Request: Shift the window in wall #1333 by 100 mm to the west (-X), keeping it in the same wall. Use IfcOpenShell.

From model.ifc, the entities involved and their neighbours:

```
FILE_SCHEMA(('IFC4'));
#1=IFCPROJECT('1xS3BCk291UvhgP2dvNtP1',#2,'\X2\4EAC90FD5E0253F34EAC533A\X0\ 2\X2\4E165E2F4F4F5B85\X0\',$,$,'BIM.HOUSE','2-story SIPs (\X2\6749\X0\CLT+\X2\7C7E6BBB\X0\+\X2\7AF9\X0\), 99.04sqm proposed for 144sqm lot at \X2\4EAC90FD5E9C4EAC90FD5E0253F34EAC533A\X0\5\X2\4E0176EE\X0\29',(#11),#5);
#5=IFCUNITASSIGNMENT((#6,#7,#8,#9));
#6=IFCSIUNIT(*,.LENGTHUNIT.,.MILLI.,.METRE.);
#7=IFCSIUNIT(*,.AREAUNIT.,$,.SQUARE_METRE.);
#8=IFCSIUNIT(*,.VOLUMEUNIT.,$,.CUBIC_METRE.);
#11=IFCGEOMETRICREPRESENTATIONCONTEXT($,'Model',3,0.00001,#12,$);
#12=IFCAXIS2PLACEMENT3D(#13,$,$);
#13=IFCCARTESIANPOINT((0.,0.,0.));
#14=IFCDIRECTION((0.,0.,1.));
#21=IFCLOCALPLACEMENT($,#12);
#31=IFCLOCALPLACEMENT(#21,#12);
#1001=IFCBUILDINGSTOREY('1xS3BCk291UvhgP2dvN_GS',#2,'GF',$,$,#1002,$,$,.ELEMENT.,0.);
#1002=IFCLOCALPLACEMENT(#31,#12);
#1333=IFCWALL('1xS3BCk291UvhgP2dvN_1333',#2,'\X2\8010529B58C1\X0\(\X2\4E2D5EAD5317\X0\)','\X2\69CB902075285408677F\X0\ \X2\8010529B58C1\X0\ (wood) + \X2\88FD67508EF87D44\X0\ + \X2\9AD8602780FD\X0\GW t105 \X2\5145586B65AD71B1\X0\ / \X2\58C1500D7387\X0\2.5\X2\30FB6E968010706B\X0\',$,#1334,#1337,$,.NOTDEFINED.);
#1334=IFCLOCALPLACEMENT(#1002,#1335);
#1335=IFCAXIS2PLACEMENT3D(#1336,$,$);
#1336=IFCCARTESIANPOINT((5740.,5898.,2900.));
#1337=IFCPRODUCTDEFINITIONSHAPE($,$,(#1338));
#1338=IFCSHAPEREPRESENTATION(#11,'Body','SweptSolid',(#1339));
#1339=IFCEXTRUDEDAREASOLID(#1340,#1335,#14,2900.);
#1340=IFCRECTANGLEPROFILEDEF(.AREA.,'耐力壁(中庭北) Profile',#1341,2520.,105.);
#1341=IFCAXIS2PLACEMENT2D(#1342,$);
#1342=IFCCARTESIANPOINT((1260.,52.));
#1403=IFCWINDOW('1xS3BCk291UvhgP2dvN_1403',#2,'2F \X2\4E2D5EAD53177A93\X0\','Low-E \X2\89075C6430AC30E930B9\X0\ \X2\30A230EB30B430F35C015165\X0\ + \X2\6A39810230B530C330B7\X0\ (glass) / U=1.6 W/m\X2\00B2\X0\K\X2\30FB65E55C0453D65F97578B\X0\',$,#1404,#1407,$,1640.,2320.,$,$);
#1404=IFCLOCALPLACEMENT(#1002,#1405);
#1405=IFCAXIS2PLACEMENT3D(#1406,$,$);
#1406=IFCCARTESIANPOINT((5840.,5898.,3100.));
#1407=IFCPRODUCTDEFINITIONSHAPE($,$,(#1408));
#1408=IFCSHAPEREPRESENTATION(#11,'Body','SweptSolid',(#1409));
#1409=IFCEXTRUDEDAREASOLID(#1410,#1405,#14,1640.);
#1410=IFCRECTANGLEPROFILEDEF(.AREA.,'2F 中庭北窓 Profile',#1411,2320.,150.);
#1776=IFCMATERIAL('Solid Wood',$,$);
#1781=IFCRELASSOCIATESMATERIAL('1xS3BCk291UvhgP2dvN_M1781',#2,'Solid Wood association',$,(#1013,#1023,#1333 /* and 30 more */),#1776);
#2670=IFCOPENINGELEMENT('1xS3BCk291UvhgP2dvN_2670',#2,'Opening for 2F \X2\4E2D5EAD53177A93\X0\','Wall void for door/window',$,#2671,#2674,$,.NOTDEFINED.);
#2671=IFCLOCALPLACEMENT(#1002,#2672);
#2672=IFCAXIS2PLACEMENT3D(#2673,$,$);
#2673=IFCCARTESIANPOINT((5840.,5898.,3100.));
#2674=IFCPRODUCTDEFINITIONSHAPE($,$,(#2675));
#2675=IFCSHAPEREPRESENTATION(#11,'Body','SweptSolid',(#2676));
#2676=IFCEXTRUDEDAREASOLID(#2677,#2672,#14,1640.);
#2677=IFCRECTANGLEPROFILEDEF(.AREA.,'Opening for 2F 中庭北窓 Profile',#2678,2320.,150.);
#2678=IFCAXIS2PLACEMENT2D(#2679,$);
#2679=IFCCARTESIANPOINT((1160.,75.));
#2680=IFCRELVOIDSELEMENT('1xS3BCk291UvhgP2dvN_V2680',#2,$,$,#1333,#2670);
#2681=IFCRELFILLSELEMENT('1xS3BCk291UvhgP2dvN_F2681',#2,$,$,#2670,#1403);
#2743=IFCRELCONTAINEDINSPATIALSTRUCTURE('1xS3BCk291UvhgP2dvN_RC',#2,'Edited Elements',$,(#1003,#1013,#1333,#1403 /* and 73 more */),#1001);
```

```python
import ifcopenshell
import ifcopenshell.api.geometry
import ifcopenshell.util.placement
import ifcopenshell.util.unit

model = ifcopenshell.open("model.ifc")
unit_scale = ifcopenshell.util.unit.calculate_unit_scale(model)

window = model.by_guid("1xS3BCk291UvhgP2dvN_1403")
opening = window.FillsVoids[0].RelatingOpeningElement
wall = opening.VoidsElements[0].RelatingBuildingElement

wall_matrix = ifcopenshell.util.placement.get_local_placement(wall.ObjectPlacement)
shift = wall_matrix[:3, 0] * -0.1 / unit_scale
before = ifcopenshell.util.placement.get_local_placement(window.ObjectPlacement)[:3, 3].copy()

# The window is not placed relative to its opening, so move both.
for product in (opening, window):
    matrix = ifcopenshell.util.placement.get_local_placement(product.ObjectPlacement)
    matrix[:3, 3] += shift
    ifcopenshell.api.geometry.edit_object_placement(model, product=product, matrix=matrix, is_si=False)

after = ifcopenshell.util.placement.get_local_placement(window.ObjectPlacement)[:3, 3]
print("window moved by", (after - before).round(3) + 0.0)

model.write("model_edited.ifc")
```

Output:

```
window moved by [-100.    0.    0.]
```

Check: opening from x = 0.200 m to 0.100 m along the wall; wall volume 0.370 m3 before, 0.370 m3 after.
